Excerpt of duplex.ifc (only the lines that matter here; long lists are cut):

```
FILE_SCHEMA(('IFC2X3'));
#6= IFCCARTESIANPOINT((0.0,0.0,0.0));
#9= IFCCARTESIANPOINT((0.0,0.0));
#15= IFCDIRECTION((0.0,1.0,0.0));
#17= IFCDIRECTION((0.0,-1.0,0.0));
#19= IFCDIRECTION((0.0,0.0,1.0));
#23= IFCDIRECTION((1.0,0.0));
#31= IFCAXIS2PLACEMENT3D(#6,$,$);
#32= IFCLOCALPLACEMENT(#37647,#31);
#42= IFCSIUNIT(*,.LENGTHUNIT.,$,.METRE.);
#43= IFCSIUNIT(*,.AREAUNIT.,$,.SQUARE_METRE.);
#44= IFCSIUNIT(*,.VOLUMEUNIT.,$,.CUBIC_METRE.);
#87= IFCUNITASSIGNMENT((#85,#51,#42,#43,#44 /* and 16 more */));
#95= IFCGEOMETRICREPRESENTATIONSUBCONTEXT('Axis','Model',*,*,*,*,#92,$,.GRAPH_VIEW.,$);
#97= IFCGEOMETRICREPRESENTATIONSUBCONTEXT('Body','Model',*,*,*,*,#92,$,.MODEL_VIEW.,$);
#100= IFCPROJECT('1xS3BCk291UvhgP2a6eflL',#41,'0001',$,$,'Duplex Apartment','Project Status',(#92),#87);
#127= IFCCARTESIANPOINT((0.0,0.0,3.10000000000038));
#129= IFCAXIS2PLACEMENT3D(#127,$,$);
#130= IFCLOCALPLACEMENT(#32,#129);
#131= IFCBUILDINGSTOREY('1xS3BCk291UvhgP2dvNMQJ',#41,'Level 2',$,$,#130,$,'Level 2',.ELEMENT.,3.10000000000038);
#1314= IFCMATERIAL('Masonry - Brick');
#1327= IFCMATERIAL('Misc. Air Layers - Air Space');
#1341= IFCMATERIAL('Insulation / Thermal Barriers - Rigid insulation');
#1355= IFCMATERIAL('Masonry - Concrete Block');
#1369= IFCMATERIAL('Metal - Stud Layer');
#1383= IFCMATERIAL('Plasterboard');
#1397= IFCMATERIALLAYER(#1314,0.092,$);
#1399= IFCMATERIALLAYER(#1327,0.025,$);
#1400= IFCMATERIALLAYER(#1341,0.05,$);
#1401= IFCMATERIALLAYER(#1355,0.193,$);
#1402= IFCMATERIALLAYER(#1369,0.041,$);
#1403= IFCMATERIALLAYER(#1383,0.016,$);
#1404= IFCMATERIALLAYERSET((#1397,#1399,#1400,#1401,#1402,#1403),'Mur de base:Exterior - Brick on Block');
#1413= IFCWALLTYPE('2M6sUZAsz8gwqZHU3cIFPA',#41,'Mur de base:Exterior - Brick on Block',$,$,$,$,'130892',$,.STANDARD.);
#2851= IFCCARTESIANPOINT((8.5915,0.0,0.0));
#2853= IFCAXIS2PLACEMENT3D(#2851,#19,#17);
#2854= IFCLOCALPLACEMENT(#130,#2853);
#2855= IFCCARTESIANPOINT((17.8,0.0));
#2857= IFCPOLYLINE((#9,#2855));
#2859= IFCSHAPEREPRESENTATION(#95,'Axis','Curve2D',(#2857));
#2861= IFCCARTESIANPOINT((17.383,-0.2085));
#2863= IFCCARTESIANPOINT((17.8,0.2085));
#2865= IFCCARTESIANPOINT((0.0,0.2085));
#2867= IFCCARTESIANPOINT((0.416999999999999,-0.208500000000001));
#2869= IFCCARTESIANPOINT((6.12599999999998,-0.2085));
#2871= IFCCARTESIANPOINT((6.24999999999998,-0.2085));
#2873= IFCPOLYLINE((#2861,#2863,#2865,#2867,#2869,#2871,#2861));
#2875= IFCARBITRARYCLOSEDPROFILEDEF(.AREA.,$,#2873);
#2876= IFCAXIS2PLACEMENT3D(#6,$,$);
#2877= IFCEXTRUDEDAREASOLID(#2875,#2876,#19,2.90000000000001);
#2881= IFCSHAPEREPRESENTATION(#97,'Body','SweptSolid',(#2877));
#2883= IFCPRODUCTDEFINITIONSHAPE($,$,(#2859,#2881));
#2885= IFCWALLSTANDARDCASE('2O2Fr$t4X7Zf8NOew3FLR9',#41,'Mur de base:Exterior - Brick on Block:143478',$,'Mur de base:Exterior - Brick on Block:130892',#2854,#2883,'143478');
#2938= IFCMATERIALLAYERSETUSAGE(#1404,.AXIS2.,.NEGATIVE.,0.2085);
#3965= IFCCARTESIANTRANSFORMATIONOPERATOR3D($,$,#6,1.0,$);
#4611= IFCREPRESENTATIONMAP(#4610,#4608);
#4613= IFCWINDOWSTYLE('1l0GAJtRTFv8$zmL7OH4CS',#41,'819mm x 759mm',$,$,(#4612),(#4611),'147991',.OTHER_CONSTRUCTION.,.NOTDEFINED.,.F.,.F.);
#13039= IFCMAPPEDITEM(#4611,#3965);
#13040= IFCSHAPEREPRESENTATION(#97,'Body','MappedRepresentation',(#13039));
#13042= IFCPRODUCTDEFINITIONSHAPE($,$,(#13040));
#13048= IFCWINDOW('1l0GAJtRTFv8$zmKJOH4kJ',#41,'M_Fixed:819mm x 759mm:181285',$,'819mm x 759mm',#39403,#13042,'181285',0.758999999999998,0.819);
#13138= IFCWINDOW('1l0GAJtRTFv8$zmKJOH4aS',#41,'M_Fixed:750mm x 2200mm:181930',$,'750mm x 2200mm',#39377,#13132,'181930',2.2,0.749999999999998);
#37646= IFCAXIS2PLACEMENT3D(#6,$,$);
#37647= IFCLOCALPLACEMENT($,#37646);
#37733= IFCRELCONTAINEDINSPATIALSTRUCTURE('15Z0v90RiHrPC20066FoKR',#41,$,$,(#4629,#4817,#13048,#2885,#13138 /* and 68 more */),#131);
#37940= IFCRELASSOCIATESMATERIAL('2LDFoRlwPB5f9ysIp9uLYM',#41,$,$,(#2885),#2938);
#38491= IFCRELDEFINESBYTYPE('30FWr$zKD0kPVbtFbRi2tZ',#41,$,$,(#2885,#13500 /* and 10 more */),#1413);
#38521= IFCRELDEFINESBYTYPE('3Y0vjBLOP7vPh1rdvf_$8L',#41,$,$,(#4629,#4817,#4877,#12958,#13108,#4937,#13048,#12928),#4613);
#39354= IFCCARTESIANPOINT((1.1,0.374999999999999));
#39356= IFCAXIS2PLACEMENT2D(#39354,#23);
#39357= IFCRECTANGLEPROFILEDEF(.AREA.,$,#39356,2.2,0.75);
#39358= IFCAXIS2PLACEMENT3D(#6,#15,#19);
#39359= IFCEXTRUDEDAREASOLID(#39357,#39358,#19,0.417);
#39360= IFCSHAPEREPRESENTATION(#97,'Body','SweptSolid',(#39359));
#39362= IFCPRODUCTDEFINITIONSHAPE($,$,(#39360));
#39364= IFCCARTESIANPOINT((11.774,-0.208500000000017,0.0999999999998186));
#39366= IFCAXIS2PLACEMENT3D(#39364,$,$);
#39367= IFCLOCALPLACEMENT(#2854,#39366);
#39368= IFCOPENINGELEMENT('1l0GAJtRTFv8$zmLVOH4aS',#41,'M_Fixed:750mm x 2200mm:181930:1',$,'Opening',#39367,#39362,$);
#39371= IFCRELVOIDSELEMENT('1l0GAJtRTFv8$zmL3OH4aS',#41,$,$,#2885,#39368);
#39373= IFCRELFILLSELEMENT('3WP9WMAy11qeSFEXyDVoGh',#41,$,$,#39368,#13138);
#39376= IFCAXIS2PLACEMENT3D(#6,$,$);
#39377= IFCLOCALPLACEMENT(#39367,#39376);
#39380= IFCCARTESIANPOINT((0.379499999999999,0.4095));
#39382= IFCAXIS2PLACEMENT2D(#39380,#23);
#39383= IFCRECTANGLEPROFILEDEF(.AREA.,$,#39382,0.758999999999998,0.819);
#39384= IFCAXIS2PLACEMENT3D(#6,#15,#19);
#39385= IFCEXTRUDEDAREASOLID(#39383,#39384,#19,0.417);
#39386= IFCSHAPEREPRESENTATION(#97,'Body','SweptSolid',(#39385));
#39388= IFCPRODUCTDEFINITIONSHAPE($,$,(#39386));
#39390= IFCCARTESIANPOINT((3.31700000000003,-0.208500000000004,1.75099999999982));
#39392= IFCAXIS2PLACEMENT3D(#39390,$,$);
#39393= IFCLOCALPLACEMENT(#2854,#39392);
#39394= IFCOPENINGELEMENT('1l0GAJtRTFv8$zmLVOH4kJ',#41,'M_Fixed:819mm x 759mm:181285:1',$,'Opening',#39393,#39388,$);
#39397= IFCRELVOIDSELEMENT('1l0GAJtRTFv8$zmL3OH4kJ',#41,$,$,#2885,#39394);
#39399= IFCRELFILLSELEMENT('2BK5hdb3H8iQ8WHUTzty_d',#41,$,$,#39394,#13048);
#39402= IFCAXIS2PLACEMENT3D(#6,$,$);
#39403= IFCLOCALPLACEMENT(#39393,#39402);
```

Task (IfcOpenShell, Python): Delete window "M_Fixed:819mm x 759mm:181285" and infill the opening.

```python
import ifcopenshell
import ifcopenshell.api.feature
import ifcopenshell.api.root
import ifcopenshell.geom
import ifcopenshell.util.shape

model = ifcopenshell.open("duplex.ifc")
settings = ifcopenshell.geom.settings()


def volume(element):
    """Net volume in cubic metres, openings subtracted."""
    shape = ifcopenshell.geom.create_shape(settings, element)
    return ifcopenshell.util.shape.get_volume(shape.geometry)


window = model.by_guid("1l0GAJtRTFv8$zmKJOH4kJ")
opening = window.FillsVoids[0].RelatingOpeningElement
wall = opening.VoidsElements[0].RelatingBuildingElement
before = volume(wall)

ifcopenshell.api.root.remove_product(model, product=window)
ifcopenshell.api.feature.remove_feature(model, feature=opening)

after = volume(wall)

print(f"wall volume {before:.3f} -> {after:.3f} m3")

model.write("duplex_v2.ifc")
```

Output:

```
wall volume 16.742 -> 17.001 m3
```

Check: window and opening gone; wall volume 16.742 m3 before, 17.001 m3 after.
